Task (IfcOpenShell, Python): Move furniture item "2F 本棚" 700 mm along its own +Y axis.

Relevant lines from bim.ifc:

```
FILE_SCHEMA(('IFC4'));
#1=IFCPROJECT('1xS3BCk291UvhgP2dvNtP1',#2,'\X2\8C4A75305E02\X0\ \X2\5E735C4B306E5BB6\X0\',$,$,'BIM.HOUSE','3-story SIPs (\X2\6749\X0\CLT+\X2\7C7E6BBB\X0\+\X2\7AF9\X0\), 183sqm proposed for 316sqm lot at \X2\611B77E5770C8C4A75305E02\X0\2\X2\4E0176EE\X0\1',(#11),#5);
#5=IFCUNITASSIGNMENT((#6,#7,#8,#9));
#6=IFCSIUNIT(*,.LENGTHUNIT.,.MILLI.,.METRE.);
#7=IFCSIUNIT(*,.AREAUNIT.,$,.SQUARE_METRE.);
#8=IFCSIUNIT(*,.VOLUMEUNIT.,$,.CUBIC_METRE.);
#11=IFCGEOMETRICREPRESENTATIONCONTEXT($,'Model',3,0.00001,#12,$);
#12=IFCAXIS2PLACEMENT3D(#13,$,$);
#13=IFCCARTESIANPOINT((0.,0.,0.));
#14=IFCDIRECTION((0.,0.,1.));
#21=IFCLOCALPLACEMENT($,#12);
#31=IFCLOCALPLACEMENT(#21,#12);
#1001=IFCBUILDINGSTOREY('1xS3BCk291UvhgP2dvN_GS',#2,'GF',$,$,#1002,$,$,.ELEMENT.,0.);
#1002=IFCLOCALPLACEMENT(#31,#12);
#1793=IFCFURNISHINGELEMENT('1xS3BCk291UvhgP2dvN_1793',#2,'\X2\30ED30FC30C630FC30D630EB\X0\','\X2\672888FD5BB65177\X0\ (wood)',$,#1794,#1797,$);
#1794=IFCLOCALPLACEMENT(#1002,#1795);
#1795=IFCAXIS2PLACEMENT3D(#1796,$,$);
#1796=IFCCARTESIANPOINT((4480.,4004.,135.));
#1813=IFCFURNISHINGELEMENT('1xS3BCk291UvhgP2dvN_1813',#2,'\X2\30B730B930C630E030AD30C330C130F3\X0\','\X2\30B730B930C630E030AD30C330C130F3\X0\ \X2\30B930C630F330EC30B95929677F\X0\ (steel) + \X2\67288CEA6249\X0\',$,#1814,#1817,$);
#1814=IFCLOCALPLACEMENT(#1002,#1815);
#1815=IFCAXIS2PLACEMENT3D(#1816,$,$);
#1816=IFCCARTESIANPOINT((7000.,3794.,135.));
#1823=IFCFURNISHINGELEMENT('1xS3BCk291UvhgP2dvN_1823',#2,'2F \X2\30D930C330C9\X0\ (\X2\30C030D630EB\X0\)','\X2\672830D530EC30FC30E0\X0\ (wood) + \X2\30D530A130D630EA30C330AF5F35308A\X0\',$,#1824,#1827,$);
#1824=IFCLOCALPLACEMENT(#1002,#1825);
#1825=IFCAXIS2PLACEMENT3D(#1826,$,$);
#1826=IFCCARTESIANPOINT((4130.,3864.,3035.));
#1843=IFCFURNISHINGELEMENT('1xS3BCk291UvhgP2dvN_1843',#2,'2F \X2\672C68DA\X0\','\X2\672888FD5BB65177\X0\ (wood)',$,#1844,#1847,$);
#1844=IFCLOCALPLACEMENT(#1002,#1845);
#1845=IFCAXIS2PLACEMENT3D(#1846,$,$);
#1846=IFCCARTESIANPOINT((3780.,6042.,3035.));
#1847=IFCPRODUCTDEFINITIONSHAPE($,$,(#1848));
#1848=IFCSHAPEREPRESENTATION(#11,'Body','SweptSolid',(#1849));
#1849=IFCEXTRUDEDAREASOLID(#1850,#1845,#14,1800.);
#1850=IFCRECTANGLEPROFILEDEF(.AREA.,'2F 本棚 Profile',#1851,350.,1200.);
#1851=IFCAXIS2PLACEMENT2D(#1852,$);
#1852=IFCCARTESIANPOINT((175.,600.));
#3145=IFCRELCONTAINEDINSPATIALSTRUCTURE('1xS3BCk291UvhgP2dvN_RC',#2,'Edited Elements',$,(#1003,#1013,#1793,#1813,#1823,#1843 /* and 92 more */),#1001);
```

```python
import ifcopenshell
import ifcopenshell.api.geometry
import ifcopenshell.util.placement
import ifcopenshell.util.unit

model = ifcopenshell.open("bim.ifc")
unit_scale = ifcopenshell.util.unit.calculate_unit_scale(model)

item = model.by_guid("1xS3BCk291UvhgP2dvN_1843")
matrix = ifcopenshell.util.placement.get_local_placement(item.ObjectPlacement)
matrix[:3, 3] += matrix[:3, 1] * 0.7 / unit_scale
ifcopenshell.api.geometry.edit_object_placement(model, product=item, matrix=matrix, is_si=False)

print(ifcopenshell.util.placement.get_local_placement(item.ObjectPlacement).round(3) + 0.0)

model.write("bim_updated.ifc")
```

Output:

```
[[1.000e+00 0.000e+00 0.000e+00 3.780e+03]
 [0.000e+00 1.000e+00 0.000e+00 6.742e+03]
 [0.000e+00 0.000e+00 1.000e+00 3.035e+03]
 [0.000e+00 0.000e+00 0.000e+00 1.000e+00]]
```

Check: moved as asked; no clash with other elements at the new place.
